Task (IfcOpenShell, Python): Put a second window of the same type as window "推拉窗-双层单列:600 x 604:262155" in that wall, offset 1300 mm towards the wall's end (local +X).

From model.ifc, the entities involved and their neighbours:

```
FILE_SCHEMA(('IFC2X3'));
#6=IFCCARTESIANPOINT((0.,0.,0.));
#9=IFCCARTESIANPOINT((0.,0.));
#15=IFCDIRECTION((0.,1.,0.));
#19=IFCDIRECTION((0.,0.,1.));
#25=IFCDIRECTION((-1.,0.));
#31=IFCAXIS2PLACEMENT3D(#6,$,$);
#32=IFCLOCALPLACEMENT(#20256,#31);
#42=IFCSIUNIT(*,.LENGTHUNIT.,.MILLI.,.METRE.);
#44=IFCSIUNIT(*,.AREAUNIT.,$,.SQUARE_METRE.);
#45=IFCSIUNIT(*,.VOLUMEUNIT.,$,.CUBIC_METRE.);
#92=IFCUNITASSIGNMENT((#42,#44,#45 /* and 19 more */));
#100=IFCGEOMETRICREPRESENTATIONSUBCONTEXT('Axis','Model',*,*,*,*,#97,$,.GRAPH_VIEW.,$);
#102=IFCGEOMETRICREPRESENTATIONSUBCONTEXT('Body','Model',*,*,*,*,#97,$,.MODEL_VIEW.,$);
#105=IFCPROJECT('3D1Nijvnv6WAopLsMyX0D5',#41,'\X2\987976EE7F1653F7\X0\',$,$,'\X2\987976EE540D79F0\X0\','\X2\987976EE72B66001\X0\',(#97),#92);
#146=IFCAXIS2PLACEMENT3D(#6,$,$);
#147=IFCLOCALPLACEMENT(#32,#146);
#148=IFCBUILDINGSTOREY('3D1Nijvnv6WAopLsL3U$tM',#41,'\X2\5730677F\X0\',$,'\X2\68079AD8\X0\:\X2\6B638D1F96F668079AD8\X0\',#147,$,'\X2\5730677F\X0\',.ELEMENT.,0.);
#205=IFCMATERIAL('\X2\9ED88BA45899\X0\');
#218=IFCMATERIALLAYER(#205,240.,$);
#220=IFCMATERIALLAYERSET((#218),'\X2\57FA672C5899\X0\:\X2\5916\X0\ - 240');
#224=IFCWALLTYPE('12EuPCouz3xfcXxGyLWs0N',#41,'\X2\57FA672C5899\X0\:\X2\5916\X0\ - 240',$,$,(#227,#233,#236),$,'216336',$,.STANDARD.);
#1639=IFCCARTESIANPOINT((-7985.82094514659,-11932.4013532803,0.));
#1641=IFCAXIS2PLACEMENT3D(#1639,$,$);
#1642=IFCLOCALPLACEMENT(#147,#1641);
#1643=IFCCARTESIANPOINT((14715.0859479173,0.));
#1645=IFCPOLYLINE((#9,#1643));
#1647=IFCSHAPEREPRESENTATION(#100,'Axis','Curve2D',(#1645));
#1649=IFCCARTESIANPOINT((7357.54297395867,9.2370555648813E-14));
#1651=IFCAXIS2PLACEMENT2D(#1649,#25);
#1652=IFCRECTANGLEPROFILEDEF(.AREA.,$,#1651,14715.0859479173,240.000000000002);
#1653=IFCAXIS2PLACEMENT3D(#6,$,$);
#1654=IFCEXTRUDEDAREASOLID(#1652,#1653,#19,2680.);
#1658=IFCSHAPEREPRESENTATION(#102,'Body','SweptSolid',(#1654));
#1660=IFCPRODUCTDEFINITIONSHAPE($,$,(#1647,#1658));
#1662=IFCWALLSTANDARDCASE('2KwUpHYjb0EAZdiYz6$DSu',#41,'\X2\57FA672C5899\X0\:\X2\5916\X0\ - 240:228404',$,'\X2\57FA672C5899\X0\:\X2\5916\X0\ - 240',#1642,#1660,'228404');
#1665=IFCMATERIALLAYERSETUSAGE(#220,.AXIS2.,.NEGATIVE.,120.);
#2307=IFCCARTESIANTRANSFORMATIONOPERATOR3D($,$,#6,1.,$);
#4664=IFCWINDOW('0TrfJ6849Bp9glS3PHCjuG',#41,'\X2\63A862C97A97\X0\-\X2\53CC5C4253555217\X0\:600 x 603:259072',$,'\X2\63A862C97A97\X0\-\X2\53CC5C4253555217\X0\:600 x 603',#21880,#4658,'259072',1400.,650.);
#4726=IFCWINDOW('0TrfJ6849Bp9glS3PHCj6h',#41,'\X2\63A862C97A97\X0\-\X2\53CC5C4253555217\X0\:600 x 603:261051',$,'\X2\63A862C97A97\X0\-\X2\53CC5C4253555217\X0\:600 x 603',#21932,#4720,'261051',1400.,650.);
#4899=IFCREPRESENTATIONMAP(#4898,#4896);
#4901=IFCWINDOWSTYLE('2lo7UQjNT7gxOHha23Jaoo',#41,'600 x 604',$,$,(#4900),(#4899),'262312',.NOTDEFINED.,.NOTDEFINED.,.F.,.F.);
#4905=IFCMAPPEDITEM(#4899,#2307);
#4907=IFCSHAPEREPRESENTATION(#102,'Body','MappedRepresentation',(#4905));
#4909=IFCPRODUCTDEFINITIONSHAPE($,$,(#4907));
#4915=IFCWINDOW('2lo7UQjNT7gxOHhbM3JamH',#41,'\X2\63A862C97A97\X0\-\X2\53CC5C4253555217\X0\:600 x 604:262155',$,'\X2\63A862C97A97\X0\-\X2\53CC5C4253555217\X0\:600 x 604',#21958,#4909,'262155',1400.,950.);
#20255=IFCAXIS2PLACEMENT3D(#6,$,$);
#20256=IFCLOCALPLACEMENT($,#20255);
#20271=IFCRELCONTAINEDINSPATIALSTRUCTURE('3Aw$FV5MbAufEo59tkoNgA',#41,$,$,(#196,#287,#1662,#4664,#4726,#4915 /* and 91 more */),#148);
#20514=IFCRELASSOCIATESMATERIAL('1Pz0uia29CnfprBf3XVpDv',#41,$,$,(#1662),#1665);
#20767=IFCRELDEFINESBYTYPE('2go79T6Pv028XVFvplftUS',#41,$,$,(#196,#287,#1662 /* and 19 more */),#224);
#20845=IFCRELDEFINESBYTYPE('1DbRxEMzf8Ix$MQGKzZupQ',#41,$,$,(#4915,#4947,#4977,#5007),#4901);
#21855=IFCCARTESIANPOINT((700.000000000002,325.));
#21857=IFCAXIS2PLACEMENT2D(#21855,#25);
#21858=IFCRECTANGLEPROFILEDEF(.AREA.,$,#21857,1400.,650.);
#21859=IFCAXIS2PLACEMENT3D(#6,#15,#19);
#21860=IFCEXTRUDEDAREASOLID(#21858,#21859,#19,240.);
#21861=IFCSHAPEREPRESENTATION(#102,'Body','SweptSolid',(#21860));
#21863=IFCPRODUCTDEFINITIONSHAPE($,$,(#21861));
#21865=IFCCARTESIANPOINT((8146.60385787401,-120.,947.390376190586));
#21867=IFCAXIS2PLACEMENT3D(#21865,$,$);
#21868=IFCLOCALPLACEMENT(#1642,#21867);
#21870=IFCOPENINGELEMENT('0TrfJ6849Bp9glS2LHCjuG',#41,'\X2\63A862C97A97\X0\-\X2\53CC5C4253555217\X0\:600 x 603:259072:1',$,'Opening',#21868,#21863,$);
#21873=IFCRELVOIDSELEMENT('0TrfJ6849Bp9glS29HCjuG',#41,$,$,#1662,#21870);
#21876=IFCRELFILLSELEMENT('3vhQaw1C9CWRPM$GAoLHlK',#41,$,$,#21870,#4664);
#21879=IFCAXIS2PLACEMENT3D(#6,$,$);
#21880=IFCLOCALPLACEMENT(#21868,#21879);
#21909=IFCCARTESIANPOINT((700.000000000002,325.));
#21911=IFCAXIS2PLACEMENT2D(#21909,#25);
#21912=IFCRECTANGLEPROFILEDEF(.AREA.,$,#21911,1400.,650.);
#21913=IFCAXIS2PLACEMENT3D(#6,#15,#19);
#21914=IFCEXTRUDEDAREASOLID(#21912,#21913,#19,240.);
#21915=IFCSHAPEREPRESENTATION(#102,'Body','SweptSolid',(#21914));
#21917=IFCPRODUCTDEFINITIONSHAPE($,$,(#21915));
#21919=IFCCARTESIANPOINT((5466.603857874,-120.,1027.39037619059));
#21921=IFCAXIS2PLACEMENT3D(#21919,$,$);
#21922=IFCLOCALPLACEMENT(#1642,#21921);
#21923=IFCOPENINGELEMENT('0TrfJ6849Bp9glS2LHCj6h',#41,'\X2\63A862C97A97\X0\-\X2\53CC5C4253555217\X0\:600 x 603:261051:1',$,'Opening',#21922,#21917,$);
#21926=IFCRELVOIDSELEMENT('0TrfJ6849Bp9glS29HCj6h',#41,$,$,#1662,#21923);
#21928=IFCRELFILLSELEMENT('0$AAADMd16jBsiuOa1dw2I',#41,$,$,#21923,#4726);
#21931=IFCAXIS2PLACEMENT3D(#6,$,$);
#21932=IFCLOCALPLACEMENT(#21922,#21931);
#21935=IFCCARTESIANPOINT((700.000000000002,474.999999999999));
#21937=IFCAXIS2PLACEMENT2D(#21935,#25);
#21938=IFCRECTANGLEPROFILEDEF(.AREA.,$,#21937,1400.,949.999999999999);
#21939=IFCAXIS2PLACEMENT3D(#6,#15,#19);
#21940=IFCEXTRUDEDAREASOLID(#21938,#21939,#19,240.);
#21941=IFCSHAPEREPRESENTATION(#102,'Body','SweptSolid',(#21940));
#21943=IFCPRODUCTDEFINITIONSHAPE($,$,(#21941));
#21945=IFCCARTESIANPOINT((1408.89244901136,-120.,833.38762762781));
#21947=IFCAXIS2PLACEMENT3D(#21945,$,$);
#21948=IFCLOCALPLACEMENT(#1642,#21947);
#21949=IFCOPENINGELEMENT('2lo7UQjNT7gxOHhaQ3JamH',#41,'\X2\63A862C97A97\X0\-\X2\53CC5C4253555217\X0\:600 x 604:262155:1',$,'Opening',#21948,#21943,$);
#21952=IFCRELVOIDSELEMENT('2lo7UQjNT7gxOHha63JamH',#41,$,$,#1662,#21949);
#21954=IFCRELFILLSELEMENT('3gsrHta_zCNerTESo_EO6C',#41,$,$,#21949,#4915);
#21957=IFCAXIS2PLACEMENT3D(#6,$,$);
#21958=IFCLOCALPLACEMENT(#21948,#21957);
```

```python
import ifcopenshell
import ifcopenshell.api.feature
import ifcopenshell.api.geometry
import ifcopenshell.api.root
import ifcopenshell.geom
import ifcopenshell.util.element
import ifcopenshell.util.placement
import ifcopenshell.util.shape

model = ifcopenshell.open("model.ifc")
settings = ifcopenshell.geom.settings()


def volume(element):
    """Net volume in cubic metres, openings subtracted."""
    shape = ifcopenshell.geom.create_shape(settings, element)
    return ifcopenshell.util.shape.get_volume(shape.geometry)


def reuse_history(source, copy):
    """copy_class also copies each property set's owner history, people and application; keep the originals."""
    for rel in copy.IsDefinedBy:
        if rel.is_a("IfcRelDefinesByProperties") and (history := rel.RelatingPropertyDefinition.OwnerHistory):
            rel.RelatingPropertyDefinition.OwnerHistory = source.OwnerHistory
            ifcopenshell.util.element.remove_deep2(model, history)


window = model.by_guid("2lo7UQjNT7gxOHhbM3JamH")
opening = window.FillsVoids[0].RelatingOpeningElement
wall = opening.VoidsElements[0].RelatingBuildingElement
before = volume(wall)
shift = ifcopenshell.util.placement.get_local_placement(wall.ObjectPlacement)[:3, 0] * 1300.0

# copy_class copies the void relationship, type, container and properties, but no geometry.
new_opening = ifcopenshell.api.root.copy_class(model, product=opening)
new_opening.Representation = ifcopenshell.util.element.copy_deep(
    model, opening.Representation, exclude=["IfcGeometricRepresentationContext", "IfcRepresentationMap"]
)
new_opening.Name = "推拉窗-双层单列:600 x 604"
new_window = ifcopenshell.api.root.copy_class(model, product=window)
new_window.Representation = ifcopenshell.util.element.copy_deep(
    model, window.Representation, exclude=["IfcGeometricRepresentationContext", "IfcRepresentationMap"]
)
new_window.Name = "推拉窗-双层单列:600 x 604"
new_window.Tag = None
reuse_history(window, new_window)
fills = ifcopenshell.api.feature.add_filling(model, opening=new_opening, element=new_window)
fills.OwnerHistory = new_window.OwnerHistory  # required in IFC2X3

for old, new in ((opening, new_opening), (window, new_window)):
    matrix = ifcopenshell.util.placement.get_local_placement(old.ObjectPlacement)
    matrix[:3, 3] += shift
    ifcopenshell.api.geometry.edit_object_placement(model, product=new, matrix=matrix, is_si=False)

after = volume(wall)

print(f"wall volume {before:.3f} -> {after:.3f} m3")

model.write("model_edited.ifc")
```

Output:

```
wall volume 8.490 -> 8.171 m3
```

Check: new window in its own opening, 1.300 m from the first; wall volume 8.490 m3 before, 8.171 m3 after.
